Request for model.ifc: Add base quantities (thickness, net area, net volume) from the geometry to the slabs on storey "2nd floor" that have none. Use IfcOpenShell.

First a look at what the model holds.

```python
import ifcopenshell
import ifcopenshell.util.element
import ifcopenshell.util.unit

model = ifcopenshell.open("model.ifc")
print(model.schema)
for unit_type in ("LENGTHUNIT", "AREAUNIT", "VOLUMEUNIT"):
    print(unit_type, ifcopenshell.util.unit.calculate_unit_scale(model, unit_type))
storey = next(s for s in model.by_type("IfcBuildingStorey") if s.Name == "2nd floor")
slabs = [e for e in ifcopenshell.util.element.get_decomposition(storey) if e.is_a("IfcSlab")]
for e in sorted(slabs, key=lambda e: e.id()):
    print(e.id(), e.is_a(), e.Name, list(ifcopenshell.util.element.get_psets(e, qtos_only=True)), sep=" | ")
```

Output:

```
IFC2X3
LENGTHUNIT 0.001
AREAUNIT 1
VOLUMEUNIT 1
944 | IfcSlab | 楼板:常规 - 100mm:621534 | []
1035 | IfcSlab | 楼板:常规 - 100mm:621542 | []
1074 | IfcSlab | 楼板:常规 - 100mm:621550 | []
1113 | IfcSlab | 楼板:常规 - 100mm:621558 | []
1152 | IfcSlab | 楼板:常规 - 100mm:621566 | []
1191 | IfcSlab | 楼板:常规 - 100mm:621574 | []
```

```python
import ifcopenshell
import ifcopenshell.api.pset
import ifcopenshell.geom
import ifcopenshell.util.element
import ifcopenshell.util.shape
import ifcopenshell.util.unit

model = ifcopenshell.open("model.ifc")
unit_scale = ifcopenshell.util.unit.calculate_unit_scale(model)
area_scale = ifcopenshell.util.unit.calculate_unit_scale(model, "AREAUNIT")
volume_scale = ifcopenshell.util.unit.calculate_unit_scale(model, "VOLUMEUNIT")
settings = ifcopenshell.geom.settings()

storey = next(s for s in model.by_type("IfcBuildingStorey") if s.Name == "2nd floor")
slabs = [e for e in ifcopenshell.util.element.get_decomposition(storey) if e.is_a("IfcSlab")]

for e in sorted(slabs, key=lambda e: e.id()):
    if ifcopenshell.util.element.get_psets(e, qtos_only=True, should_inherit=False):
        continue
    # Geometry comes back in metres, in the element's own axes.
    shape = ifcopenshell.geom.create_shape(settings, e)
    values = {
        "Width": ifcopenshell.util.shape.get_z(shape.geometry) / unit_scale,
        "NetArea": ifcopenshell.util.shape.get_footprint_area(shape.geometry) / area_scale,
        "NetVolume": ifcopenshell.util.shape.get_volume(shape.geometry) / volume_scale,
    }
    qto = ifcopenshell.api.pset.add_qto(model, product=e, name="BaseQuantities")
    ifcopenshell.api.pset.edit_qto(model, qto=qto, properties=values)
    print(e.id(), {k: round(v, 3) for k, v in values.items()})

model.write("model_edited.ifc")
```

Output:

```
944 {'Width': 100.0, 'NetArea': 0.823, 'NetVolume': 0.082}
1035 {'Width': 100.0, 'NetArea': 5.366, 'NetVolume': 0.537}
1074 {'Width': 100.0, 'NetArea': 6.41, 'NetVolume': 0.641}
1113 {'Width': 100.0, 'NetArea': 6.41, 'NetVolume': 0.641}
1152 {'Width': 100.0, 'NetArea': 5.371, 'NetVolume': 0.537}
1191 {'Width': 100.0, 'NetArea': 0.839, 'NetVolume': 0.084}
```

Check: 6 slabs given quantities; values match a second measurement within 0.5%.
